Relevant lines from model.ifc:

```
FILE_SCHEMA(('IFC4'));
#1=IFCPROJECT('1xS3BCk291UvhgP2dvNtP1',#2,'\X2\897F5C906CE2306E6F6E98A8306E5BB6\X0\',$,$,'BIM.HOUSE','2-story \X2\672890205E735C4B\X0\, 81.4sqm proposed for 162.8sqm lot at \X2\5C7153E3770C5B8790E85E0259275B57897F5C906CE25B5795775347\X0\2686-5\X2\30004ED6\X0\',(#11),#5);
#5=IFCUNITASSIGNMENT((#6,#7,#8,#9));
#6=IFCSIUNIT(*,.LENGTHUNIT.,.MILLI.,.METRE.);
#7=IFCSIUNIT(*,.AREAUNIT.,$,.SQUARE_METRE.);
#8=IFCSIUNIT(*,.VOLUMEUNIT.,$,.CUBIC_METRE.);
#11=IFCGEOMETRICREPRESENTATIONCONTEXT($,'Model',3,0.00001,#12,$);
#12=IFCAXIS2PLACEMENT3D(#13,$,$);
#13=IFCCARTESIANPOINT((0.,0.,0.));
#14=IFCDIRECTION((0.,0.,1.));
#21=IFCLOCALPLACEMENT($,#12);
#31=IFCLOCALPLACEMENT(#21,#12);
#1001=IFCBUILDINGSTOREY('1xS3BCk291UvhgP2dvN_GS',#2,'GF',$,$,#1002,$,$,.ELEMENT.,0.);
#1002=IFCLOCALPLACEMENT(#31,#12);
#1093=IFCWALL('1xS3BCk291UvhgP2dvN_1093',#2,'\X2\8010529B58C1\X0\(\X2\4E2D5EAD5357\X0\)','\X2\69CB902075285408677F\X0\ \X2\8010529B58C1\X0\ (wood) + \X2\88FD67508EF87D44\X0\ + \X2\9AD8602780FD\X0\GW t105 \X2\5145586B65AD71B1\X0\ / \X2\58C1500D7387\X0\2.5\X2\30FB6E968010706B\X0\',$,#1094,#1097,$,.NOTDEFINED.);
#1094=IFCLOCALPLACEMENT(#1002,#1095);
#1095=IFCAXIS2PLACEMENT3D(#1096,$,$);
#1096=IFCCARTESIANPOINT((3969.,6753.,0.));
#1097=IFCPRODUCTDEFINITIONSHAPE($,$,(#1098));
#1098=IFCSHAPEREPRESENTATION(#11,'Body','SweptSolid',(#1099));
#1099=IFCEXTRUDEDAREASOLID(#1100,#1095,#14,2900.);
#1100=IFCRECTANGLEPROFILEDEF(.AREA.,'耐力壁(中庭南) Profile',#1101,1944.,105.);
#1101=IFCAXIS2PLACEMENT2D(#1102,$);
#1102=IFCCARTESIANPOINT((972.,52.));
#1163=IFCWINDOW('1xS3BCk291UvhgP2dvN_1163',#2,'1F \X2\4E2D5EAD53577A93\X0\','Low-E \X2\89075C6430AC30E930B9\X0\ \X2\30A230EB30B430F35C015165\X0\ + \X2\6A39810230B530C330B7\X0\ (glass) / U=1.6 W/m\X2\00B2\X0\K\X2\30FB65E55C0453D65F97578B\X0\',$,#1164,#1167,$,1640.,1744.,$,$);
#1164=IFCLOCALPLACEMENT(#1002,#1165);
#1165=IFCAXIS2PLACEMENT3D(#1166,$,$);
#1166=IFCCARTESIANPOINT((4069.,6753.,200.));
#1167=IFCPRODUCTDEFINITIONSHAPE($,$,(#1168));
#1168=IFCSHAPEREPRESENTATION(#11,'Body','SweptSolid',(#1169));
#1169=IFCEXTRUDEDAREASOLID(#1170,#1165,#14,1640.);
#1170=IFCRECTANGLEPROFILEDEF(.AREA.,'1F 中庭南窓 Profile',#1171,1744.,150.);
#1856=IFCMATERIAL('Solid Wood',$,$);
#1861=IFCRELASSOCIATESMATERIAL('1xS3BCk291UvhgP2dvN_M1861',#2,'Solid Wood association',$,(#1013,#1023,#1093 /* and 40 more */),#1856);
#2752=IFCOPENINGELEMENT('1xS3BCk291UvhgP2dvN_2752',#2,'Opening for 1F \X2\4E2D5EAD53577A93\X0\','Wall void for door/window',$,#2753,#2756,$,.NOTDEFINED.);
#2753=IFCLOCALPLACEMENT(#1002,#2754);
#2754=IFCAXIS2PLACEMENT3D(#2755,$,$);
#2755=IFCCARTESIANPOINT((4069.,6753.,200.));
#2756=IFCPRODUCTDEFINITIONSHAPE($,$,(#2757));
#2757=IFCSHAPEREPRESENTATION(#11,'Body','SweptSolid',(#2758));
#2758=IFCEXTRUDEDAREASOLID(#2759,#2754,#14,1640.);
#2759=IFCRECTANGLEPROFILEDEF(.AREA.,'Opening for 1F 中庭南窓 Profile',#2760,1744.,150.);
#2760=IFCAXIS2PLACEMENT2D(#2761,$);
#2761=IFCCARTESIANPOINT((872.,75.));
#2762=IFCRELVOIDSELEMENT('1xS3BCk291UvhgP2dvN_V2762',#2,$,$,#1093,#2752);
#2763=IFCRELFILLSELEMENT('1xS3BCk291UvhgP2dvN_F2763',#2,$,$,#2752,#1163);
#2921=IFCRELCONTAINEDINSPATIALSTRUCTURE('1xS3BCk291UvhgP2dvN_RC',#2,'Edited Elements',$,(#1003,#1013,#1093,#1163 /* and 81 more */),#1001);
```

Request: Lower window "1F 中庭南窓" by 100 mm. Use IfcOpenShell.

```python
import numpy as np
import ifcopenshell
import ifcopenshell.api.geometry
import ifcopenshell.util.placement
import ifcopenshell.util.unit

model = ifcopenshell.open("model.ifc")
unit_scale = ifcopenshell.util.unit.calculate_unit_scale(model)

window = model.by_guid("1xS3BCk291UvhgP2dvN_1163")
opening = window.FillsVoids[0].RelatingOpeningElement
dz = -100.0

shift = np.array([0.0, 0.0, dz])
# The window is not placed relative to its opening, so move both.
for product in (opening, window):
    matrix = ifcopenshell.util.placement.get_local_placement(product.ObjectPlacement)
    matrix[:3, 3] += shift
    ifcopenshell.api.geometry.edit_object_placement(model, product=product, matrix=matrix, is_si=False)

print(f"moved by {dz * unit_scale:+.3f} m")

model.write("model_updated.ifc")
```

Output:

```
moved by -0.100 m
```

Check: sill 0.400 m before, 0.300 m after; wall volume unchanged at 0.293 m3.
